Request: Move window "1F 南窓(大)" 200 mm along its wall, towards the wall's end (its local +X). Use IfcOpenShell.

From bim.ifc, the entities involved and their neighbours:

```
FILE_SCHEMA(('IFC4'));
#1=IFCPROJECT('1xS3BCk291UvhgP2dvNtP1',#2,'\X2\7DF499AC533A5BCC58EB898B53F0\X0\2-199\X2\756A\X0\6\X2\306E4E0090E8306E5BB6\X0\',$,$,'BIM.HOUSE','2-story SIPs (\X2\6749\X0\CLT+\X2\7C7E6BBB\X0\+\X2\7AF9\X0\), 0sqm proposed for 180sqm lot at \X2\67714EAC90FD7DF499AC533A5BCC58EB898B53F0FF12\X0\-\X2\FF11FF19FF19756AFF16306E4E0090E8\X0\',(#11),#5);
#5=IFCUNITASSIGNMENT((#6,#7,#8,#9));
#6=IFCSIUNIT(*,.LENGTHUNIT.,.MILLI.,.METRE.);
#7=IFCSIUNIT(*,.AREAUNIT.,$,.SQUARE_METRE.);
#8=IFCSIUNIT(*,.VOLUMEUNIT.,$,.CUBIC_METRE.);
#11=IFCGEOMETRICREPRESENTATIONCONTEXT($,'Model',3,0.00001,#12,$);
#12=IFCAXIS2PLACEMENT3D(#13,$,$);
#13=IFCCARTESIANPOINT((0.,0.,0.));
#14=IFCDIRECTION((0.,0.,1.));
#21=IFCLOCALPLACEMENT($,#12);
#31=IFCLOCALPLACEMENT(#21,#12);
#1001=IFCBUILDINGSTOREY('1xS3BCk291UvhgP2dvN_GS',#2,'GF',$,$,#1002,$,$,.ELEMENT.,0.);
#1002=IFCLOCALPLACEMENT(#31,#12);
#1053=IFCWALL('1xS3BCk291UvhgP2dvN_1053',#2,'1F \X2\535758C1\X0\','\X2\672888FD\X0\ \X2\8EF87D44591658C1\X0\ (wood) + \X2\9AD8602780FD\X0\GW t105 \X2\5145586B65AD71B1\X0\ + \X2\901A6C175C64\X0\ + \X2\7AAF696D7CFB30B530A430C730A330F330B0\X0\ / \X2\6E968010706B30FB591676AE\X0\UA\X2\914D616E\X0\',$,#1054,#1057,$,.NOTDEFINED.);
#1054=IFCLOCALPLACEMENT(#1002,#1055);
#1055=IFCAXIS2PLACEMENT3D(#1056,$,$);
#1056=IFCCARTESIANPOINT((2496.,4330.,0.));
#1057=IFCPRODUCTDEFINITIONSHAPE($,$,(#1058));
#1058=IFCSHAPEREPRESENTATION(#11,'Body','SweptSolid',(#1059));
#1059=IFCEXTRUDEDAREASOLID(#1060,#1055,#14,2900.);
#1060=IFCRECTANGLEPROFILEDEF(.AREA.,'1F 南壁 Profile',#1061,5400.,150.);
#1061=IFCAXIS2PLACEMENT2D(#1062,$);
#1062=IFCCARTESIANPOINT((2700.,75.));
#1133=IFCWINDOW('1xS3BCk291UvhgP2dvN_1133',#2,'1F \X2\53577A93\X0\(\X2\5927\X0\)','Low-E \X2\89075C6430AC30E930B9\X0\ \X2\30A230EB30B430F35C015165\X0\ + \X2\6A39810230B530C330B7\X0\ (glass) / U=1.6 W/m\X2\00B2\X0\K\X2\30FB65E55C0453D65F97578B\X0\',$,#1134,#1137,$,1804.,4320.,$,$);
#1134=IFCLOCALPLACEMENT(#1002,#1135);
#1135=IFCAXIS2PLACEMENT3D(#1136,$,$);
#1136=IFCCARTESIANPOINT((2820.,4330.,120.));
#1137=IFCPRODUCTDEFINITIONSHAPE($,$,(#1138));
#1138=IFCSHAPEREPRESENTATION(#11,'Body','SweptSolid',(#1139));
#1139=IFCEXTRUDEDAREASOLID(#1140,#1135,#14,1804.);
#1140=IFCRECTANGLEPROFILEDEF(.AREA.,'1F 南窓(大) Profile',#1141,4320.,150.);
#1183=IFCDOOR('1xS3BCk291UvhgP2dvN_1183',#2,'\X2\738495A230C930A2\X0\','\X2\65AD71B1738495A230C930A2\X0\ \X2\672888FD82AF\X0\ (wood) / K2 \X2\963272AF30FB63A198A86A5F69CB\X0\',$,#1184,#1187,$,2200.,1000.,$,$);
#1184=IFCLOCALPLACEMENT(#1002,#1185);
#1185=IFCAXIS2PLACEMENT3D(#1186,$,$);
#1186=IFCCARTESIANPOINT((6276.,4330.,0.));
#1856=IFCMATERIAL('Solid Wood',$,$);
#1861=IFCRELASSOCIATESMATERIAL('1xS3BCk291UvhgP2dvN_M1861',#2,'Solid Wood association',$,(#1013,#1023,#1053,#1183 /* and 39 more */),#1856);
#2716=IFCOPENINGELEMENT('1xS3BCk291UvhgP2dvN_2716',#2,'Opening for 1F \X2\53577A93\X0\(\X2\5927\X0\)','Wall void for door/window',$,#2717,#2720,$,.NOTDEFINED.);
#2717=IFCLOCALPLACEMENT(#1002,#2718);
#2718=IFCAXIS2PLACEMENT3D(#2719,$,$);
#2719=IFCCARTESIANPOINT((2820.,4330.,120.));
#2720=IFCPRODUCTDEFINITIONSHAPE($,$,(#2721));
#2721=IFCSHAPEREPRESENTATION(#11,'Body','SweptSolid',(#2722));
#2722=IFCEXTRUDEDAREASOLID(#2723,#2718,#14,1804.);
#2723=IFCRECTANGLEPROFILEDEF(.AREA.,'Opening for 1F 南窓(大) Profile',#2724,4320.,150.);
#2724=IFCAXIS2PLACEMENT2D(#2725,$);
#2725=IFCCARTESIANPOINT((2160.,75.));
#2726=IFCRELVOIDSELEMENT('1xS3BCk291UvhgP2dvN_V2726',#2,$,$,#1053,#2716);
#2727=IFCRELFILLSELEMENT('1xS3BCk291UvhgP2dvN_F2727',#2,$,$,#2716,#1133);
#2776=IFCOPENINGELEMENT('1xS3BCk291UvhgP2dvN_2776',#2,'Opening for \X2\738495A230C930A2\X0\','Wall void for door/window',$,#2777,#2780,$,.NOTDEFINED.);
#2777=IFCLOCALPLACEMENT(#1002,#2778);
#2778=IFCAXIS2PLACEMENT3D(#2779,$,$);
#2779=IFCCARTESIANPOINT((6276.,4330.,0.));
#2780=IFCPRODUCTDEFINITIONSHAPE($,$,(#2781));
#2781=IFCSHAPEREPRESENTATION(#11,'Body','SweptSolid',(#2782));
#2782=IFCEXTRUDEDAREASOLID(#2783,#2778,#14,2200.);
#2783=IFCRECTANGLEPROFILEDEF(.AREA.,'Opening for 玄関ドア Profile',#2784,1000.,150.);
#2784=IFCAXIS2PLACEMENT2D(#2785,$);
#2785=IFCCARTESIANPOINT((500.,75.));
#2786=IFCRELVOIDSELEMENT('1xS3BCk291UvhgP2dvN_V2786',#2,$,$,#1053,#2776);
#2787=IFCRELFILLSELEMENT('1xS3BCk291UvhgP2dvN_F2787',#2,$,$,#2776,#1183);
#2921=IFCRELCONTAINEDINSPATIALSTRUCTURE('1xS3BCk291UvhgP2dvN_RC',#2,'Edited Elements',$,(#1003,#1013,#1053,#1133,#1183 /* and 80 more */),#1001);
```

```python
import ifcopenshell
import ifcopenshell.api.geometry
import ifcopenshell.util.placement

model = ifcopenshell.open("bim.ifc")

window = model.by_guid("1xS3BCk291UvhgP2dvN_1133")
opening = window.FillsVoids[0].RelatingOpeningElement
wall = opening.VoidsElements[0].RelatingBuildingElement

wall_matrix = ifcopenshell.util.placement.get_local_placement(wall.ObjectPlacement)
shift = wall_matrix[:3, 0] * 200.0
before = ifcopenshell.util.placement.get_local_placement(window.ObjectPlacement)[:3, 3].copy()

# The window is not placed relative to its opening, so move both.
for product in (opening, window):
    matrix = ifcopenshell.util.placement.get_local_placement(product.ObjectPlacement)
    matrix[:3, 3] += shift
    ifcopenshell.api.geometry.edit_object_placement(model, product=product, matrix=matrix, is_si=False)

after = ifcopenshell.util.placement.get_local_placement(window.ObjectPlacement)[:3, 3]
print("window moved by", (after - before).round(3) + 0.0)

model.write("bim_updated.ifc")
```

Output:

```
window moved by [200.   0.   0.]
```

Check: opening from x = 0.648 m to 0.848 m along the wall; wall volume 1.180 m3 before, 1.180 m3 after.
